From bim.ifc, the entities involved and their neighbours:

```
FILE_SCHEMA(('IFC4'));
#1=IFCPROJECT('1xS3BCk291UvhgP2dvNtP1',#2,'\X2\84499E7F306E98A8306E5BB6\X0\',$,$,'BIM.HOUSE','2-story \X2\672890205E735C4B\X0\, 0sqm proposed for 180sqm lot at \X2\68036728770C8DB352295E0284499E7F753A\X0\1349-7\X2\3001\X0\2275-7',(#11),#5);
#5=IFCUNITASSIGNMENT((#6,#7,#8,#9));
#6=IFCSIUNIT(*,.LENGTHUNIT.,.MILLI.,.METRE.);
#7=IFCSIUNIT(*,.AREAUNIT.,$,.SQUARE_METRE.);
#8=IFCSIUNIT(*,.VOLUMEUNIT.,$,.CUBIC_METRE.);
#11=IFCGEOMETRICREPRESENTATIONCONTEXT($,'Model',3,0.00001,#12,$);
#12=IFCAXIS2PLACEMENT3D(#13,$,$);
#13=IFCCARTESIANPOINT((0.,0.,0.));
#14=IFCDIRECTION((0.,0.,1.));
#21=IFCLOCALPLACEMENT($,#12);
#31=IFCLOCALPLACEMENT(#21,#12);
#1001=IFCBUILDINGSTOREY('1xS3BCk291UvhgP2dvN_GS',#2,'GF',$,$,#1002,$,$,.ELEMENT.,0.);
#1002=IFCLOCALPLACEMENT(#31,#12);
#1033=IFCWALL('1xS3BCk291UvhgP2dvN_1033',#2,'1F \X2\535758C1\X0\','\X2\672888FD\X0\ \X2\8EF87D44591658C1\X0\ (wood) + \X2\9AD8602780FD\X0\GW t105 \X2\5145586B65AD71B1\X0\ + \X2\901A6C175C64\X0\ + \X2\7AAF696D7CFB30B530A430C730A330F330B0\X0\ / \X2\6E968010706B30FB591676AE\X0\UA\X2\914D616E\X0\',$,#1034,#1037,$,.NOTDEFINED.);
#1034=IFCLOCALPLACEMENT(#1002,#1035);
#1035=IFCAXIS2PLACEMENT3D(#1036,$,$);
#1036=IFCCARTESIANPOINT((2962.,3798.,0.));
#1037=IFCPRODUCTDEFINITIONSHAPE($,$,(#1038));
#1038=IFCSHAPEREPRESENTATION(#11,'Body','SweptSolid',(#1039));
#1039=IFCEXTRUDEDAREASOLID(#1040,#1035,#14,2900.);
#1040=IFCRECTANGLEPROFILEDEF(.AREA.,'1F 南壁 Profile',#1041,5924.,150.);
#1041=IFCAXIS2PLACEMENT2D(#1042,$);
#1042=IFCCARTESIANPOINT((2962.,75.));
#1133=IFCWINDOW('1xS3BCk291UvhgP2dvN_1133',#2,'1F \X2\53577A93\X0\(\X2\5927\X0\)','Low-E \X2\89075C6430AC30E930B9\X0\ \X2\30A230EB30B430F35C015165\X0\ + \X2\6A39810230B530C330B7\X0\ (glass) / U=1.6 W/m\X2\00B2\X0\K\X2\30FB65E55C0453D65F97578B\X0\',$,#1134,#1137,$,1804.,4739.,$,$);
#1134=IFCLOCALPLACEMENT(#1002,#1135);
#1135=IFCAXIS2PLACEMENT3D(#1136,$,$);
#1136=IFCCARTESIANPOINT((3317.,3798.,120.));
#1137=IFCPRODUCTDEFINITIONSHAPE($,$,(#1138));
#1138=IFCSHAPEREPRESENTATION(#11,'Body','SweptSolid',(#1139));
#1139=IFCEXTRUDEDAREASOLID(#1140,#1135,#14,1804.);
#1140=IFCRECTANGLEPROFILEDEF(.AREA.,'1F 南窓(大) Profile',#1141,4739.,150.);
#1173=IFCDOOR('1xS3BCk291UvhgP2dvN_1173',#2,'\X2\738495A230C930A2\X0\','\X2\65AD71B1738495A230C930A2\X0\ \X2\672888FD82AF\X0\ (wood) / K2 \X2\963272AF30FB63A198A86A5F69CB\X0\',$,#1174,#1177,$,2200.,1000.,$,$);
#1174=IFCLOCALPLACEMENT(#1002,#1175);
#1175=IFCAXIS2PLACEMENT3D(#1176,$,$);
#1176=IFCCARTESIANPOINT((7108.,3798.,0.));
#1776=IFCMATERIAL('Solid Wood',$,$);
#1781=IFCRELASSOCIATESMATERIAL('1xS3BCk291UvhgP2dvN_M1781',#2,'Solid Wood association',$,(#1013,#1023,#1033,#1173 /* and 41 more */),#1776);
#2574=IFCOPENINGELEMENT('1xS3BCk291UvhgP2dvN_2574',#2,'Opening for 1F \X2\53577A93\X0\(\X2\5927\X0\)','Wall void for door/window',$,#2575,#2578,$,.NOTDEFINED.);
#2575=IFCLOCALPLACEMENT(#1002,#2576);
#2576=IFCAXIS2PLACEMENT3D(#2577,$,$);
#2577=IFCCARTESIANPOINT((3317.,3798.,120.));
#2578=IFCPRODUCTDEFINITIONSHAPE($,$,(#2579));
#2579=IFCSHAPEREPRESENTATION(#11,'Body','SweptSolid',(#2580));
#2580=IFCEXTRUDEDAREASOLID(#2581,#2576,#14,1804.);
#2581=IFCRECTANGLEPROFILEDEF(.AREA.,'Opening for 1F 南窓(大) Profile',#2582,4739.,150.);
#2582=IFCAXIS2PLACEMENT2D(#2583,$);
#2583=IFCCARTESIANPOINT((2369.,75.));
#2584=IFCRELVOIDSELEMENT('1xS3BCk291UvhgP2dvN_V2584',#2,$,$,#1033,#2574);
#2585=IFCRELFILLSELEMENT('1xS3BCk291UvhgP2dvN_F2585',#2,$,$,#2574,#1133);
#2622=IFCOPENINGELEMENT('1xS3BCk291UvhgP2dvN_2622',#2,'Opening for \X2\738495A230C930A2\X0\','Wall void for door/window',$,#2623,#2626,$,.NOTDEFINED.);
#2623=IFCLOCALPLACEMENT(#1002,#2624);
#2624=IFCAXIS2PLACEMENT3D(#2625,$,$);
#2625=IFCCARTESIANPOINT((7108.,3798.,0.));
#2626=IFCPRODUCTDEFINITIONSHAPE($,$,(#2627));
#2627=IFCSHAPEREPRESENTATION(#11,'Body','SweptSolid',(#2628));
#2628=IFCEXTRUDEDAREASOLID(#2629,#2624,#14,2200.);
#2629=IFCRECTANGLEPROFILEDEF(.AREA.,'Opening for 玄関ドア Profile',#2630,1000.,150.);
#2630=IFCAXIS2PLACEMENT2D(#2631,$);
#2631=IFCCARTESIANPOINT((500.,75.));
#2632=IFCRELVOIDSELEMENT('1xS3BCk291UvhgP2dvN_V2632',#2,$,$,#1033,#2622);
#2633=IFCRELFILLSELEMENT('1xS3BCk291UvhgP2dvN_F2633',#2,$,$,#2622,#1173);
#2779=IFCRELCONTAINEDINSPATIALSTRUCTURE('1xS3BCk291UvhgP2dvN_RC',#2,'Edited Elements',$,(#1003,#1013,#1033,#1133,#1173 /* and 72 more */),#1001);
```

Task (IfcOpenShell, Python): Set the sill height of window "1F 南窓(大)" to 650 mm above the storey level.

```python
import numpy as np
import ifcopenshell
import ifcopenshell.api.geometry
import ifcopenshell.geom
import ifcopenshell.util.element
import ifcopenshell.util.placement
import ifcopenshell.util.shape
import ifcopenshell.util.unit

model = ifcopenshell.open("bim.ifc")
unit_scale = ifcopenshell.util.unit.calculate_unit_scale(model)

window = model.by_guid("1xS3BCk291UvhgP2dvN_1133")
opening = window.FillsVoids[0].RelatingOpeningElement
storey = ifcopenshell.util.element.get_container(window, ifc_class="IfcBuildingStorey")
level = ifcopenshell.util.placement.get_local_placement(storey.ObjectPlacement)[2, 3]

# The opening's origin need not be at the sill, so measure its lowest point.
shape = ifcopenshell.geom.create_shape(ifcopenshell.geom.settings(), opening)
bottom = ifcopenshell.util.shape.get_shape_bottom_elevation(shape, shape.geometry) / unit_scale
dz = level + 0.65 / unit_scale - bottom

shift = np.array([0.0, 0.0, dz])
# The window is not placed relative to its opening, so move both.
for product in (opening, window):
    matrix = ifcopenshell.util.placement.get_local_placement(product.ObjectPlacement)
    matrix[:3, 3] += shift
    ifcopenshell.api.geometry.edit_object_placement(model, product=product, matrix=matrix, is_si=False)

print(f"moved by {dz * unit_scale:+.3f} m")

model.write("bim-out.ifc")
```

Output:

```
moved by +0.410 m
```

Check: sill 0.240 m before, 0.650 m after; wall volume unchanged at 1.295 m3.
